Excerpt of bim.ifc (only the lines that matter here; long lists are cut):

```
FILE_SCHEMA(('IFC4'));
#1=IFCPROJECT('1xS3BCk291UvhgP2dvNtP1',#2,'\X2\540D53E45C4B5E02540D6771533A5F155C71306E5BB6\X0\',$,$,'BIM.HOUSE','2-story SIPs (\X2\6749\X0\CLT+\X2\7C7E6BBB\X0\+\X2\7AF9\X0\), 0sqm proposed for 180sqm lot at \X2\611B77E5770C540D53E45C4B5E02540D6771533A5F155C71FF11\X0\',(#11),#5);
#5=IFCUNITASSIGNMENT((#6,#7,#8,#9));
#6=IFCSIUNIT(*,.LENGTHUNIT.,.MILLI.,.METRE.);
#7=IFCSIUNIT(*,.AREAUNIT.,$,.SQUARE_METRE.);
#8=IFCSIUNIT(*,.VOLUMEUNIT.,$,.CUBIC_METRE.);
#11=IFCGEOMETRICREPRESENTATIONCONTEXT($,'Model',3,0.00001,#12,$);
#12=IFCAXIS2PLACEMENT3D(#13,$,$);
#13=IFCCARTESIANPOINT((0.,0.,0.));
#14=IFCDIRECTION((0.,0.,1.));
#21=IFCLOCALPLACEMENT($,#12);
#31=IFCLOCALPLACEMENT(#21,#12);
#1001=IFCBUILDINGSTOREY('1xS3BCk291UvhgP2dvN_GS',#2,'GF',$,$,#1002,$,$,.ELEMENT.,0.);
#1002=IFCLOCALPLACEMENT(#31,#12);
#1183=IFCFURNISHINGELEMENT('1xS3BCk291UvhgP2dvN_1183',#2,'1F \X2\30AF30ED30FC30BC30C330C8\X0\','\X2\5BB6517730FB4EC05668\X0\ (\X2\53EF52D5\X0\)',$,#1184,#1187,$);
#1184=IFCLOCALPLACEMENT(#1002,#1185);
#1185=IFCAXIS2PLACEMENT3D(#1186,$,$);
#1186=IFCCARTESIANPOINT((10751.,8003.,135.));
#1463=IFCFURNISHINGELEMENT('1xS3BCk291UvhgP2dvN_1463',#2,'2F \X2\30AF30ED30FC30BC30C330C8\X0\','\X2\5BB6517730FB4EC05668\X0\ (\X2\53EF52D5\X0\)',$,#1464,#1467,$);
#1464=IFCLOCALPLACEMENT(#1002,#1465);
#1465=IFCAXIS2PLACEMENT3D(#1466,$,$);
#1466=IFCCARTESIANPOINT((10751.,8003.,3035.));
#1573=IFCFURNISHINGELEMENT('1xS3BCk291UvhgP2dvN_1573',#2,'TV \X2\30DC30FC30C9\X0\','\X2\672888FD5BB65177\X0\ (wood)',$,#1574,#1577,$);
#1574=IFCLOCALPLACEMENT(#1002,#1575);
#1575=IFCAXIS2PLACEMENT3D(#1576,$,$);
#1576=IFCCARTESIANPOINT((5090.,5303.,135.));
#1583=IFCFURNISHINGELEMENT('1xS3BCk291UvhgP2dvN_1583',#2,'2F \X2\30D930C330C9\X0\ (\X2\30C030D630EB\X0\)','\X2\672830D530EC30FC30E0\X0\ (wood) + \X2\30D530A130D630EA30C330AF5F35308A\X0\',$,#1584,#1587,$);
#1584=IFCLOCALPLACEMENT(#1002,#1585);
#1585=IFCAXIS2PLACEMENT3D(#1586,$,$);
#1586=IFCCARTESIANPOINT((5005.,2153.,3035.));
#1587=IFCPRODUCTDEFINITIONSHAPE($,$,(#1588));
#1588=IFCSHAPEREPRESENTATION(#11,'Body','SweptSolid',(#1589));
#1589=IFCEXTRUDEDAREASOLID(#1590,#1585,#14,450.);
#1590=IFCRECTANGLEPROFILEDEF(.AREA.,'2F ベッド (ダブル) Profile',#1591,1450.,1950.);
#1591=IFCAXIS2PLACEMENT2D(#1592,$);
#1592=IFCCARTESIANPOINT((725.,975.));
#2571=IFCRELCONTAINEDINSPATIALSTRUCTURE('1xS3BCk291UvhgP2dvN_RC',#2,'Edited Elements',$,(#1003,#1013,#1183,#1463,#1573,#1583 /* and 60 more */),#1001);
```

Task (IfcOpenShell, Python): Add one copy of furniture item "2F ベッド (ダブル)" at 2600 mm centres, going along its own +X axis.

```python
import ifcopenshell
import ifcopenshell.api.geometry
import ifcopenshell.api.root
import ifcopenshell.util.element
import ifcopenshell.util.placement

model = ifcopenshell.open("bim.ifc")


def reuse_history(source, copy):
    """copy_class also copies each property set's owner history, people and application; keep the originals."""
    for rel in copy.IsDefinedBy:
        if rel.is_a("IfcRelDefinesByProperties") and (history := rel.RelatingPropertyDefinition.OwnerHistory):
            rel.RelatingPropertyDefinition.OwnerHistory = source.OwnerHistory
            ifcopenshell.util.element.remove_deep2(model, history)


source = model.by_guid("1xS3BCk291UvhgP2dvN_1583")
base = ifcopenshell.util.placement.get_local_placement(source.ObjectPlacement)
step = base[:3, 0] * 2600.0

for i in range(1, 2):
    copy = ifcopenshell.api.root.copy_class(model, product=source)
    copy.Representation = ifcopenshell.util.element.copy_deep(
        model, source.Representation, exclude=["IfcGeometricRepresentationContext", "IfcRepresentationMap"]
    )
    reuse_history(source, copy)
    matrix = base.copy()
    matrix[:3, 3] += i * step
    print("added at", matrix[:3, 3].round(3) + 0.0)
    ifcopenshell.api.geometry.edit_object_placement(model, product=copy, matrix=matrix, is_si=False)

model.write("bim_edited.ifc")
```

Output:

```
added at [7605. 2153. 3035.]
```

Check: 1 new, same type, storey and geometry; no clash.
